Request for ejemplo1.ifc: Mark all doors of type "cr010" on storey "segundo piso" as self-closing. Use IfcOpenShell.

First a look at what the model holds.

```python
import ifcopenshell
import ifcopenshell.util.element

model = ifcopenshell.open("ejemplo1.ifc")
print(model.schema)
storey = next(s for s in model.by_type("IfcBuildingStorey") if s.Name == "segundo piso")
doors = [e for e in ifcopenshell.util.element.get_decomposition(storey) if e.is_a("IfcDoor")]
seen = {}
for e in doors:
    element_type = ifcopenshell.util.element.get_type(e)
    key = (element_type.Name if element_type != e and element_type else None, ifcopenshell.util.element.get_pset(e, "Pset_DoorCommon", "SelfClosing"))
    seen[key] = seen.get(key, 0) + 1
for (name, value), count in sorted(seen.items(), key=str):
    print(count, "x", name, "|", value)
```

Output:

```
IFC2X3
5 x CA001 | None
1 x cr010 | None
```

```python
import ifcopenshell
import ifcopenshell.api.pset
import ifcopenshell.util.element

model = ifcopenshell.open("ejemplo1.ifc")

storey = next(s for s in model.by_type("IfcBuildingStorey") if s.Name == "segundo piso")
doors = [e for e in ifcopenshell.util.element.get_decomposition(storey) if e.is_a("IfcDoor")]

count = 0
for e in doors:
    element_type = ifcopenshell.util.element.get_type(e)
    if element_type in (None, e) or element_type.Name != "cr010":
        continue
    # add_pset returns the element's existing set when there is one.
    pset = ifcopenshell.api.pset.add_pset(model, product=e, name="Pset_DoorCommon")
    ifcopenshell.api.pset.edit_pset(model, pset=pset, properties={"SelfClosing": True})
    count += 1

print(count, "doors updated")

model.write("ejemplo1-out.ifc")
```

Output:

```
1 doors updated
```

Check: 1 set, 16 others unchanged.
